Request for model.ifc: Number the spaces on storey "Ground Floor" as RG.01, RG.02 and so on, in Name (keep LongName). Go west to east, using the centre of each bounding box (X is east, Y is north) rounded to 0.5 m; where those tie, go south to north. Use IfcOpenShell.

First a look at what the model holds.

```python
import ifcopenshell
import ifcopenshell.util.element
import ifcopenshell.util.placement

model = ifcopenshell.open("model.ifc")
print(model.schema)
storey = next(s for s in model.by_type("IfcBuildingStorey") if s.Name == "Ground Floor")
spaces = [e for e in ifcopenshell.util.element.get_decomposition(storey) if e.is_a("IfcSpace")]
for e in sorted(spaces, key=lambda e: e.id()):
    origin = ifcopenshell.util.placement.get_local_placement(e.ObjectPlacement)[:3, 3]
    print(e.id(), e.Name, e.LongName, origin.round(2) + 0.0, sep=" | ")
```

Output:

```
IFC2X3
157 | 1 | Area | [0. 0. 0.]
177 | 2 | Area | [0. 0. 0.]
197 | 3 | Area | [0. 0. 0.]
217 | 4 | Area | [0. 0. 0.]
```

```python
import ifcopenshell
import ifcopenshell.geom
import ifcopenshell.util.element
import ifcopenshell.util.shape

model = ifcopenshell.open("model.ifc")
settings = ifcopenshell.geom.settings()
settings.set("use-world-coords", True)


def centre(element):
    shape = ifcopenshell.geom.create_shape(settings, element)
    return ifcopenshell.util.shape.get_bbox_centroid(shape.geometry)


storey = next(s for s in model.by_type("IfcBuildingStorey") if s.Name == "Ground Floor")
spaces = [e for e in ifcopenshell.util.element.get_decomposition(storey) if e.is_a("IfcSpace")]

# Insertion points can sit at a corner or the storey origin, so sort by the geometry (in metres).
centres = {e: centre(e) for e in spaces}
spaces.sort(key=lambda e: (round(centres[e][0] / 0.5), centres[e][1]))

for i, e in enumerate(spaces, start=1):
    number = f"RG.{i:02d}"
    e.Name = number
    print(e.id(), number)

model.write("model_edited.ifc")
```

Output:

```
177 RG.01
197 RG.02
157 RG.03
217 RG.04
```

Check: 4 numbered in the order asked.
